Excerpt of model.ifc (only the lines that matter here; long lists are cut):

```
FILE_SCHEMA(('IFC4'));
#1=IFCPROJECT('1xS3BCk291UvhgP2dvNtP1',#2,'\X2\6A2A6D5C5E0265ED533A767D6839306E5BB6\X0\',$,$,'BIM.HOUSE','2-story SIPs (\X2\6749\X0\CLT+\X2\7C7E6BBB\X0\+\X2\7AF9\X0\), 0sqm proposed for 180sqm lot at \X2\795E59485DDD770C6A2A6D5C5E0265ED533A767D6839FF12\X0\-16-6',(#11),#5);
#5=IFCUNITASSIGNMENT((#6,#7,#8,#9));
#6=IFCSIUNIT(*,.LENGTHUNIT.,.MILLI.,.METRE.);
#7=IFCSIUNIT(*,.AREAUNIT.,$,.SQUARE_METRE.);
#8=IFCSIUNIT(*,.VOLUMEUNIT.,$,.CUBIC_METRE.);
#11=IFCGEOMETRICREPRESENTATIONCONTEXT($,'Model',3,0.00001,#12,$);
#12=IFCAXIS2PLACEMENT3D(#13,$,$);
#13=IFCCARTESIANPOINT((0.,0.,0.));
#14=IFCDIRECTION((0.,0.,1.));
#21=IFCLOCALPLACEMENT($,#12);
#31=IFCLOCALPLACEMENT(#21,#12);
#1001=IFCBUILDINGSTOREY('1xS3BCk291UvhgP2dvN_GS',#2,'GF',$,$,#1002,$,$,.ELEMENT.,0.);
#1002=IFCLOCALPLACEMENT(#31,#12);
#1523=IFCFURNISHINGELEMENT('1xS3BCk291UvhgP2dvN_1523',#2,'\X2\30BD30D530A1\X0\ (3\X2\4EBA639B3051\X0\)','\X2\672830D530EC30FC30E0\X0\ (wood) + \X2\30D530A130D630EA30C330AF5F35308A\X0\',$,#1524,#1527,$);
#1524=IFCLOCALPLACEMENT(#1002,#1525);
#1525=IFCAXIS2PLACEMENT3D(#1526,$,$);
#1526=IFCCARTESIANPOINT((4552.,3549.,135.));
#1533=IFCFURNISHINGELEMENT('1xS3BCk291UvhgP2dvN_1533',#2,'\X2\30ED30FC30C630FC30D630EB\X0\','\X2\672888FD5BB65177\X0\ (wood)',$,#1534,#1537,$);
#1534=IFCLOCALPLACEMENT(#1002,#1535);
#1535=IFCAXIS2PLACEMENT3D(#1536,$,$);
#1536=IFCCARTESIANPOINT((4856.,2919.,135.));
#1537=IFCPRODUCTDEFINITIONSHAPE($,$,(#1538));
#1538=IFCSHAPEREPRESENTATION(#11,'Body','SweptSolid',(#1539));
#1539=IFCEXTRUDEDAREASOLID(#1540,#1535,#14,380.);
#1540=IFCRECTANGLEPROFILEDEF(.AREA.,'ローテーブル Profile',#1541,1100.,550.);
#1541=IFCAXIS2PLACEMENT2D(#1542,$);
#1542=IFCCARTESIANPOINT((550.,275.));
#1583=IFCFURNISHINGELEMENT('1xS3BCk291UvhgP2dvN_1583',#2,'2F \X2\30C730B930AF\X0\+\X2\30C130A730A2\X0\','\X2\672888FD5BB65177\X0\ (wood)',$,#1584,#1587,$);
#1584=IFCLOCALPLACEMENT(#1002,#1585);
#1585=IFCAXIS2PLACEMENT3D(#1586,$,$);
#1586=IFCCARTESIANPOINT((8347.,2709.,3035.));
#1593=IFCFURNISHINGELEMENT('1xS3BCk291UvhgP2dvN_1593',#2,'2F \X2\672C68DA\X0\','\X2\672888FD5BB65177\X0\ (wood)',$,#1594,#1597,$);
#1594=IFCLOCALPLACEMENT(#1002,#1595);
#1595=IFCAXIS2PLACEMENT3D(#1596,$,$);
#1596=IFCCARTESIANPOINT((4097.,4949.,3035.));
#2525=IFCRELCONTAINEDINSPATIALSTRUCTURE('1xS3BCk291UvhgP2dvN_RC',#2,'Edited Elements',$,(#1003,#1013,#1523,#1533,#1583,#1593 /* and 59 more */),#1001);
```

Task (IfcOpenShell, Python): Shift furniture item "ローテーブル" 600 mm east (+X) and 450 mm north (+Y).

```python
import ifcopenshell
import ifcopenshell.api.geometry
import ifcopenshell.util.placement

model = ifcopenshell.open("model.ifc")

item = model.by_guid("1xS3BCk291UvhgP2dvN_1533")
matrix = ifcopenshell.util.placement.get_local_placement(item.ObjectPlacement)
matrix[0, 3] += 600.0
matrix[1, 3] += 450.0
ifcopenshell.api.geometry.edit_object_placement(model, product=item, matrix=matrix, is_si=False)

print(ifcopenshell.util.placement.get_local_placement(item.ObjectPlacement).round(3) + 0.0)

model.write("model_rev.ifc")
```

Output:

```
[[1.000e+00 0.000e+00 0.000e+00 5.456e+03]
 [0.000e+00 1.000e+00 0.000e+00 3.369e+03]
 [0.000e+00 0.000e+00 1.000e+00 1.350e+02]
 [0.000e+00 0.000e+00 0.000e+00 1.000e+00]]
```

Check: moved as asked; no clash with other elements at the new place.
